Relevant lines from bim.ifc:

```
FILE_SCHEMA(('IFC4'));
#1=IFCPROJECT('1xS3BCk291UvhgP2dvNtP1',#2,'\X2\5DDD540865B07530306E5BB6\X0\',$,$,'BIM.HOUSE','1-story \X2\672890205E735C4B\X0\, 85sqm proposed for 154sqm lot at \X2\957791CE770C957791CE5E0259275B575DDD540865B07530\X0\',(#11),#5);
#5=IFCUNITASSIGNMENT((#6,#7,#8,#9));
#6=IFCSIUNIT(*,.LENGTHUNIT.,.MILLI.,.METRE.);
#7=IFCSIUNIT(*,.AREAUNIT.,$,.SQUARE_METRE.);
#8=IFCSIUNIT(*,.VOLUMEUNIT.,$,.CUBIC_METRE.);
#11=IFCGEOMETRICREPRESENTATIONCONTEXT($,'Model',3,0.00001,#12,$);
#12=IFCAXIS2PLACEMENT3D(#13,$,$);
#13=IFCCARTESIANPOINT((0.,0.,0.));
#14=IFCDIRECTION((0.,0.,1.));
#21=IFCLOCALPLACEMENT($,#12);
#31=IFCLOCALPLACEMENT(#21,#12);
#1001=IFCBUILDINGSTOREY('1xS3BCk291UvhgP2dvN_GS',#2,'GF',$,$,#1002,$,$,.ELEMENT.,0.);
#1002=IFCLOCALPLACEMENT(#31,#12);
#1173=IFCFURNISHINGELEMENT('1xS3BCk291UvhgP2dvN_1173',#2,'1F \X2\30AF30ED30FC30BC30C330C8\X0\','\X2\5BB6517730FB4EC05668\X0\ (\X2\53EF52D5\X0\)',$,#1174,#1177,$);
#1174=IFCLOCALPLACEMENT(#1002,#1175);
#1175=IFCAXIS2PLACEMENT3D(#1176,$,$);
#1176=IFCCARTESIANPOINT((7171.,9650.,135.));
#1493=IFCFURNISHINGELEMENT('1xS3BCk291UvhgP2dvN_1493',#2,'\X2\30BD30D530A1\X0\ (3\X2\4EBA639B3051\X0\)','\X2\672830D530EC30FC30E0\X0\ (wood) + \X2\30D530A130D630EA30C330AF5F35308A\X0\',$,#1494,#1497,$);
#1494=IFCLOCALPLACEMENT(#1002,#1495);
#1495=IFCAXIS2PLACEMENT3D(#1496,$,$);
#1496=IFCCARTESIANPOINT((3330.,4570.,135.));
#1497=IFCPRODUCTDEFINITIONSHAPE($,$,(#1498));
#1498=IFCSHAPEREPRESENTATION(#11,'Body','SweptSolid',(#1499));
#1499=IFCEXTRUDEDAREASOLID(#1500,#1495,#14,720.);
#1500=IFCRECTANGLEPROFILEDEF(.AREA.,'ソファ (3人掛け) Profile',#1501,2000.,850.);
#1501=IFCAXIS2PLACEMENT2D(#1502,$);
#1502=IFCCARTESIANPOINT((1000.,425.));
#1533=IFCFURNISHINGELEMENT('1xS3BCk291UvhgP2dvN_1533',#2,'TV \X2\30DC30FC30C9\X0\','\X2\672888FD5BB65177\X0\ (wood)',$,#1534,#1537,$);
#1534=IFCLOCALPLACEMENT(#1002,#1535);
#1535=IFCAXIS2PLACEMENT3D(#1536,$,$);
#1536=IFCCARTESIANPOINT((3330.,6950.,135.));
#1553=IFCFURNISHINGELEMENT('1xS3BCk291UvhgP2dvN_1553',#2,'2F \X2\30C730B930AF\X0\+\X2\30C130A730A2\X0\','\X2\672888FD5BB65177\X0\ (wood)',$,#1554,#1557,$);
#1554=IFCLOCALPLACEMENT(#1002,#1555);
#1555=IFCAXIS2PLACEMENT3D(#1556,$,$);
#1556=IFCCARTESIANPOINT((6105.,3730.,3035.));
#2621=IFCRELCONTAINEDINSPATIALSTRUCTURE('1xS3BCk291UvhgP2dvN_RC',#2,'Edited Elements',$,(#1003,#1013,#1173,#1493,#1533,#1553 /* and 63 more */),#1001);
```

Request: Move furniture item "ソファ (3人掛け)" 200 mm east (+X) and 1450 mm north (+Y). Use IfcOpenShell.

```python
import ifcopenshell
import ifcopenshell.api.geometry
import ifcopenshell.util.placement
import ifcopenshell.util.unit

model = ifcopenshell.open("bim.ifc")
unit_scale = ifcopenshell.util.unit.calculate_unit_scale(model)

item = model.by_id(1493)
matrix = ifcopenshell.util.placement.get_local_placement(item.ObjectPlacement)
matrix[0, 3] += 0.2 / unit_scale
matrix[1, 3] += 1.45 / unit_scale
ifcopenshell.api.geometry.edit_object_placement(model, product=item, matrix=matrix, is_si=False)

print(ifcopenshell.util.placement.get_local_placement(item.ObjectPlacement).round(3) + 0.0)

model.write("bim_updated.ifc")
```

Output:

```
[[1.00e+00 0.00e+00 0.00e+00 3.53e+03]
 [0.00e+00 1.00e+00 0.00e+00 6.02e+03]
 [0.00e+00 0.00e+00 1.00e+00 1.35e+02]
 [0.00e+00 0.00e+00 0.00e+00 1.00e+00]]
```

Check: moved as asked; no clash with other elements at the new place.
